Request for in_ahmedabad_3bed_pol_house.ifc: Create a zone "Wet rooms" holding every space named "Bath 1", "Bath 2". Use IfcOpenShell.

First a look at what the model holds.

```python
import ifcopenshell

model = ifcopenshell.open("in_ahmedabad_3bed_pol_house.ifc")
print(model.schema)
seen = {}
for space in model.by_type("IfcSpace"):
    seen[space.LongName] = seen.get(space.LongName, 0) + 1
for name, count in sorted(seen.items(), key=str):
    print(count, "x", name)
print("zones:", [z.Name for z in model.by_type("IfcZone")][:20])
```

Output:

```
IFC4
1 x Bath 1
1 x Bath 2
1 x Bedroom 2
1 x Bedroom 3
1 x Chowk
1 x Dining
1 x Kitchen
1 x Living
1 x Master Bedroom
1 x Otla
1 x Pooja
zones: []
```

```python
import ifcopenshell
import ifcopenshell.api.group
import ifcopenshell.api.root

model = ifcopenshell.open("in_ahmedabad_3bed_pol_house.ifc")

names = {"Bath 1", "Bath 2"}
spaces = [s for s in model.by_type("IfcSpace") if s.LongName in names]

zone = ifcopenshell.api.root.create_entity(model, ifc_class="IfcZone", name="Wet rooms")
ifcopenshell.api.group.assign_group(model, products=spaces, group=zone)
print(len(spaces), "spaces in", zone.Name)

model.write("in_ahmedabad_3bed_pol_house_rev.ifc")
```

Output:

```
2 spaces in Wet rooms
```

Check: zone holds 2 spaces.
